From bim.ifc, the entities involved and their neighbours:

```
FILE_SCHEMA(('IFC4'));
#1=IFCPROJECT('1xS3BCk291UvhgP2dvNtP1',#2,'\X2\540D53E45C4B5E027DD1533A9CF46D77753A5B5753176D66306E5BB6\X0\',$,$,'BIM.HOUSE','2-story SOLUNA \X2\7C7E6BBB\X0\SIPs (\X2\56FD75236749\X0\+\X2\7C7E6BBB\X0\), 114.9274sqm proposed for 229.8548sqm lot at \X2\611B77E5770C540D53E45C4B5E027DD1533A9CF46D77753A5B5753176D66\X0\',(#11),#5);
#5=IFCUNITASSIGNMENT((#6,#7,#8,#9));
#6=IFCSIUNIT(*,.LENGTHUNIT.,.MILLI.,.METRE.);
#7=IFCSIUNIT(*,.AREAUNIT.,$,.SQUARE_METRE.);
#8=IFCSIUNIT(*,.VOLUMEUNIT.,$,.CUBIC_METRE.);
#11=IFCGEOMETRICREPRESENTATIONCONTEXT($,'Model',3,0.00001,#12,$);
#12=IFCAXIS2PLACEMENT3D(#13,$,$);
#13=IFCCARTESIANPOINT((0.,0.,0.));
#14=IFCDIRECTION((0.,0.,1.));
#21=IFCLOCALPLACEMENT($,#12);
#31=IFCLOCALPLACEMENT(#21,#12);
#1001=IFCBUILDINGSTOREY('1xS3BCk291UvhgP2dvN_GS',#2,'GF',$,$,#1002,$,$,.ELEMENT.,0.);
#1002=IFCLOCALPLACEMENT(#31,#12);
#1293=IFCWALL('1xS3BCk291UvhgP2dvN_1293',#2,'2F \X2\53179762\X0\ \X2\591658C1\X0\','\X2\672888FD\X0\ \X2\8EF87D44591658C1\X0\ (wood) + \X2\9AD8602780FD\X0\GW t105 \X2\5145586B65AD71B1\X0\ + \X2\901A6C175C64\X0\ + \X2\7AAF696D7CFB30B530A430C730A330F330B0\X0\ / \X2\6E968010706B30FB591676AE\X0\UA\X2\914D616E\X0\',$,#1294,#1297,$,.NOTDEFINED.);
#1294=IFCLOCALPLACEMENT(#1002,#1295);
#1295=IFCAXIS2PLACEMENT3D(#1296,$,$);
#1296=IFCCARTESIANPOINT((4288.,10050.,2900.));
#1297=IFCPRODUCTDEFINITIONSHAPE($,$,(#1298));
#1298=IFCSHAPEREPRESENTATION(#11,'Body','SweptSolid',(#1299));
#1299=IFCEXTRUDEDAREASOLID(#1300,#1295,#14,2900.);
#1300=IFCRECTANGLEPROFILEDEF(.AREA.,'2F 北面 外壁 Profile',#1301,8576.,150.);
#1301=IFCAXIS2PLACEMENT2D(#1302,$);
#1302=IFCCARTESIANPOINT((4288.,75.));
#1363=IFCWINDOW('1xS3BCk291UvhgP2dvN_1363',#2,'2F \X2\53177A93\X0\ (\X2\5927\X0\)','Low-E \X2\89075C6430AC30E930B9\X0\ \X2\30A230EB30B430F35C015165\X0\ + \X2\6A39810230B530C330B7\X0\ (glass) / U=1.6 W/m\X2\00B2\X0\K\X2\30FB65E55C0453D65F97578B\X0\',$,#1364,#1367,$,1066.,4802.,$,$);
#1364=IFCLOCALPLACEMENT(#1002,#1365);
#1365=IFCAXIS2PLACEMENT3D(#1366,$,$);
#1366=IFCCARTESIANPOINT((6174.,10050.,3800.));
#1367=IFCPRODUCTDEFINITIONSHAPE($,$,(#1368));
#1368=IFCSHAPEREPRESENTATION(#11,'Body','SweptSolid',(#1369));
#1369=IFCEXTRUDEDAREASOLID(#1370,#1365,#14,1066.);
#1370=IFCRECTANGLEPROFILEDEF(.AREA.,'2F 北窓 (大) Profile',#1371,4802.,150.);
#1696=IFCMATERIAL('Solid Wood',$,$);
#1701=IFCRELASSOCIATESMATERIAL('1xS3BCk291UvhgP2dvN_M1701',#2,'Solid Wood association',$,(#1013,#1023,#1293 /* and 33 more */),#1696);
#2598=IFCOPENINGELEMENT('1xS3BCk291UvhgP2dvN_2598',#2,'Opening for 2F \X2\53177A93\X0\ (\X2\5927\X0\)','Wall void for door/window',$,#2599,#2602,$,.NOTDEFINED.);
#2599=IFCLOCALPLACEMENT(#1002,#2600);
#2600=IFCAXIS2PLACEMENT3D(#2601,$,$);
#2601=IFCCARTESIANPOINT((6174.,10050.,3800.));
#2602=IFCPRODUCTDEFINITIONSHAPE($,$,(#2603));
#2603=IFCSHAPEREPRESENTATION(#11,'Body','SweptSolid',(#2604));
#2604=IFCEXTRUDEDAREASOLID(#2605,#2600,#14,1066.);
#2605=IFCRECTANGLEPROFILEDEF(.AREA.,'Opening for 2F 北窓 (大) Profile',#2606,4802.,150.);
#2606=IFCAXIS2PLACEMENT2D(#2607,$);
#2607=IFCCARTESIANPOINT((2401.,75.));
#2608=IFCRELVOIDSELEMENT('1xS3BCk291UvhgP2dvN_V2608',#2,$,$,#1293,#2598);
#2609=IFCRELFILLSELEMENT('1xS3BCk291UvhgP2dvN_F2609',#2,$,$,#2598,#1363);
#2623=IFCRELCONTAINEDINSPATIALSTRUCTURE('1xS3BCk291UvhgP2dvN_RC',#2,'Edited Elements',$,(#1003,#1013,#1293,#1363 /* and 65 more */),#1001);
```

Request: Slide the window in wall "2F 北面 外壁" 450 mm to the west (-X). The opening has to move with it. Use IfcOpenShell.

```python
import ifcopenshell
import ifcopenshell.api.geometry
import ifcopenshell.util.placement
import ifcopenshell.util.unit

model = ifcopenshell.open("bim.ifc")
unit_scale = ifcopenshell.util.unit.calculate_unit_scale(model)

window = model.by_guid("1xS3BCk291UvhgP2dvN_1363")
opening = window.FillsVoids[0].RelatingOpeningElement
wall = opening.VoidsElements[0].RelatingBuildingElement

wall_matrix = ifcopenshell.util.placement.get_local_placement(wall.ObjectPlacement)
shift = wall_matrix[:3, 0] * -0.45 / unit_scale
before = ifcopenshell.util.placement.get_local_placement(window.ObjectPlacement)[:3, 3].copy()

# The window is not placed relative to its opening, so move both.
for product in (opening, window):
    matrix = ifcopenshell.util.placement.get_local_placement(product.ObjectPlacement)
    matrix[:3, 3] += shift
    ifcopenshell.api.geometry.edit_object_placement(model, product=product, matrix=matrix, is_si=False)

after = ifcopenshell.util.placement.get_local_placement(window.ObjectPlacement)[:3, 3]
print("window moved by", (after - before).round(3) + 0.0)

model.write("bim_updated.ifc")
```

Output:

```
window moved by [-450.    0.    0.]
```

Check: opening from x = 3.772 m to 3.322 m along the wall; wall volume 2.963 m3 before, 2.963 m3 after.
